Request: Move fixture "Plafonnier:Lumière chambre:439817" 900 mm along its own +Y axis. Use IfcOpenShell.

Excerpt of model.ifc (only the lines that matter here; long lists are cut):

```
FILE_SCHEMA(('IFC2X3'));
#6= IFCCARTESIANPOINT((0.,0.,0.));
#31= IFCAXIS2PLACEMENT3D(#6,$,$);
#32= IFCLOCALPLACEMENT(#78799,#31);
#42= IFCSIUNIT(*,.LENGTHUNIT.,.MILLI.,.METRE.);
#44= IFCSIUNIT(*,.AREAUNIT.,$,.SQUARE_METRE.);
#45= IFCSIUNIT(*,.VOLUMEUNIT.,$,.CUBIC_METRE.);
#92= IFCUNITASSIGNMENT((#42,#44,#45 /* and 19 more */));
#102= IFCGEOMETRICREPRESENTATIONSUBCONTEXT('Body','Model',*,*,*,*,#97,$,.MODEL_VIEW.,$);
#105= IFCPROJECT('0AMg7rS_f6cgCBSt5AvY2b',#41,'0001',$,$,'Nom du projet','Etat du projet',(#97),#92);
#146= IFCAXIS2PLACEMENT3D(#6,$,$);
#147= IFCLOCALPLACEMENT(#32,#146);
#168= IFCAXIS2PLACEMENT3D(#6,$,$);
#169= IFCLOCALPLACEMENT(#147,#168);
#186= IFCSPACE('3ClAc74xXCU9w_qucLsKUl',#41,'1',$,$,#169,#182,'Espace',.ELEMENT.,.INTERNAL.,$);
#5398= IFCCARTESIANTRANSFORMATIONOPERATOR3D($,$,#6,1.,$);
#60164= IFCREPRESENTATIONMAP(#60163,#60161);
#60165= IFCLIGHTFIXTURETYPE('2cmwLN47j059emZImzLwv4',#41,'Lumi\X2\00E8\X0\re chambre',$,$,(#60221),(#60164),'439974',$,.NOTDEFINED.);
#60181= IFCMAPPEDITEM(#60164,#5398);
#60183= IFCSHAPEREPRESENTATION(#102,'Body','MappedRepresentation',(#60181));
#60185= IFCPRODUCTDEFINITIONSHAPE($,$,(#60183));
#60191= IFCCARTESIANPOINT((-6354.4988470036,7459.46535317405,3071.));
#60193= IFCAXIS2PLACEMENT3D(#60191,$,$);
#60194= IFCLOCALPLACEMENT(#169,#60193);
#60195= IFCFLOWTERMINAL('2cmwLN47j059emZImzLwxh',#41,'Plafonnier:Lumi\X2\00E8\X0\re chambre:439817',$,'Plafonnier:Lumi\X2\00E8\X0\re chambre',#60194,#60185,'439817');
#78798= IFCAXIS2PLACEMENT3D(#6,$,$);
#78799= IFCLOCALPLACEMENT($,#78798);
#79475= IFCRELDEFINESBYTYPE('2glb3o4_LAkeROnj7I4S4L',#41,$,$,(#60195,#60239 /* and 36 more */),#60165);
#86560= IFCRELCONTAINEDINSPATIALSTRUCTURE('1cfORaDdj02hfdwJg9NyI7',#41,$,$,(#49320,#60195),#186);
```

```python
import ifcopenshell
import ifcopenshell.api.geometry
import ifcopenshell.util.placement

model = ifcopenshell.open("model.ifc")

item = model.by_guid("2cmwLN47j059emZImzLwxh")
matrix = ifcopenshell.util.placement.get_local_placement(item.ObjectPlacement)
matrix[:3, 3] += matrix[:3, 1] * 900.0
ifcopenshell.api.geometry.edit_object_placement(model, product=item, matrix=matrix, is_si=False)

print(ifcopenshell.util.placement.get_local_placement(item.ObjectPlacement).round(3) + 0.0)

model.write("model_edited.ifc")
```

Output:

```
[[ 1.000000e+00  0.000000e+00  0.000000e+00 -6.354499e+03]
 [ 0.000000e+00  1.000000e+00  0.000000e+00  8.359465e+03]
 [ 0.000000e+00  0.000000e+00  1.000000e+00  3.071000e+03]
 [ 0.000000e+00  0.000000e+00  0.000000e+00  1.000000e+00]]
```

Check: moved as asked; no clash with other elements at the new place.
